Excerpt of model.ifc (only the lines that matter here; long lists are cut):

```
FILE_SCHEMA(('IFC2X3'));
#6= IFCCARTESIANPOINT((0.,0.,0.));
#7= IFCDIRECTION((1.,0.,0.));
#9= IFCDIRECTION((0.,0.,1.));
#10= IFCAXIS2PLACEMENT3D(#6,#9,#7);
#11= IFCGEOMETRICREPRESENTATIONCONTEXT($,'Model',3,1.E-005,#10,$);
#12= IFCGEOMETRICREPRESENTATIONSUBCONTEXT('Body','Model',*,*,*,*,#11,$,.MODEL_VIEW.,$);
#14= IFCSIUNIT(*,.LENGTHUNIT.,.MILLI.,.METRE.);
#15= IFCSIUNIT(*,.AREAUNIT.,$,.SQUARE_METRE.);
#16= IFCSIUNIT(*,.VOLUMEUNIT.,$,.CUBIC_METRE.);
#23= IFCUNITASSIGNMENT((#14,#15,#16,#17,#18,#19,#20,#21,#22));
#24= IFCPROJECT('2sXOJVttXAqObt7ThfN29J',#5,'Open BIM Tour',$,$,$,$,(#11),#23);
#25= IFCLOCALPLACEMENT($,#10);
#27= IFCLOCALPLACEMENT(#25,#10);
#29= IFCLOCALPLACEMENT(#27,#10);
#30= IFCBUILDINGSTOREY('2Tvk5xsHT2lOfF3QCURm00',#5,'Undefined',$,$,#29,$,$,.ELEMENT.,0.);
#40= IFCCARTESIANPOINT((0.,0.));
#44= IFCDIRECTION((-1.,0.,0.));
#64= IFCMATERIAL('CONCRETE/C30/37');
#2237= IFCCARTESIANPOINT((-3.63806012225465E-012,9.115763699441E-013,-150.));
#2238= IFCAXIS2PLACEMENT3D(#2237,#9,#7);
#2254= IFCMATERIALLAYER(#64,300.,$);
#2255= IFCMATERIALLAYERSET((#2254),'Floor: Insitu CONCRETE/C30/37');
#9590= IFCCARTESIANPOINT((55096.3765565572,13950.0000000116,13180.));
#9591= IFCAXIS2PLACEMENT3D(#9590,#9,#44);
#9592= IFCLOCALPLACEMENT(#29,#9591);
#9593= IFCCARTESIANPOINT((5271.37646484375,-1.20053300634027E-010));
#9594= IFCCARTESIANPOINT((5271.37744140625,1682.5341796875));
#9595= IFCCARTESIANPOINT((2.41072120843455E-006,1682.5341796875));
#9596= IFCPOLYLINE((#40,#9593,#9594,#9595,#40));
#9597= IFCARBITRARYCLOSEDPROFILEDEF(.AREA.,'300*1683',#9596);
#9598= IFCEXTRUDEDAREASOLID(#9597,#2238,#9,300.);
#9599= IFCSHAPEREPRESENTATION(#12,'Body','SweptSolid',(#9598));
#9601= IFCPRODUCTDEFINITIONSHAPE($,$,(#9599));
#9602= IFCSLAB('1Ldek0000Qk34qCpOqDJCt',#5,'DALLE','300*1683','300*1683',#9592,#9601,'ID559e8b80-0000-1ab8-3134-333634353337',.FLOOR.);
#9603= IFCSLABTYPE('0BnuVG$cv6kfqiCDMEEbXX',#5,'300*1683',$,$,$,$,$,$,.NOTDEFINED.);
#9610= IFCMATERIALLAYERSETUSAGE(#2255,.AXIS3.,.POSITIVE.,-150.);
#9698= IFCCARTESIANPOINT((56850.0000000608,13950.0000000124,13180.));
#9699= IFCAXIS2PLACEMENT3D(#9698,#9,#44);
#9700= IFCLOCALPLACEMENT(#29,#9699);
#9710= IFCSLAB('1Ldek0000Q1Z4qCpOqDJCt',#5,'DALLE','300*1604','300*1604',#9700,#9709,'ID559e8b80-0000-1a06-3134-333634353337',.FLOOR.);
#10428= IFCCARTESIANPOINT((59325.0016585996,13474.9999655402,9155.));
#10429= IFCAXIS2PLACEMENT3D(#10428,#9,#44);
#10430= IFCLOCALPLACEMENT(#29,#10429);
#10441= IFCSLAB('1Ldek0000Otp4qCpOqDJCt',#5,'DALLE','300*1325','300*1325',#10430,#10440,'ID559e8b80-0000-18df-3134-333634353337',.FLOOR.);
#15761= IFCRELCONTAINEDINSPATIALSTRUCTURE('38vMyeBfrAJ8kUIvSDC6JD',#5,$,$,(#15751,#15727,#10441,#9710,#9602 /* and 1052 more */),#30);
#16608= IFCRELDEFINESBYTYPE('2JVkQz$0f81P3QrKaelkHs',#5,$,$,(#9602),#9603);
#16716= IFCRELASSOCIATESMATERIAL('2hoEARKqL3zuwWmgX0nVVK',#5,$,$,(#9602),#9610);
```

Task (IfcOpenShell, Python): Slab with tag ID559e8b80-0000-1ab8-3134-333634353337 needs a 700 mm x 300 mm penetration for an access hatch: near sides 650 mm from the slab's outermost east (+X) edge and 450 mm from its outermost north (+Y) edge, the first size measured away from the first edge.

```python
import numpy as np
import ifcopenshell
import ifcopenshell.api.feature
import ifcopenshell.api.geometry
import ifcopenshell.api.root
import ifcopenshell.geom
import ifcopenshell.util.placement
import ifcopenshell.util.representation
import ifcopenshell.util.shape
import ifcopenshell.util.unit

model = ifcopenshell.open("model.ifc")
unit_scale = ifcopenshell.util.unit.calculate_unit_scale(model)
settings = ifcopenshell.geom.settings()


def volume(element):
    """Net volume in cubic metres, openings subtracted."""
    shape = ifcopenshell.geom.create_shape(settings, element)
    return ifcopenshell.util.shape.get_volume(shape.geometry)


slab = model.by_guid("1Ldek0000Qk34qCpOqDJCt")
before = volume(slab)

# Extent in the slab's own axes, in metres. The edges named are its -X and -Y sides.
slab_shape = ifcopenshell.geom.create_shape(settings, slab)
vertices = ifcopenshell.util.shape.get_vertices(slab_shape.geometry)
x_min, y_min, bottom = vertices.min(axis=0)
top = vertices[:, 2].max()

opening = ifcopenshell.api.root.create_entity(model, ifc_class="IfcOpeningElement", name="Access hatch opening")
context = ifcopenshell.util.representation.get_context(model, "Model", "Body", "MODEL_VIEW")
width, depth = 0.7, 0.3
outline = [(0.0, 0.0), (width, 0.0), (width, depth), (0.0, depth), (0.0, 0.0)]
# Overshoot both faces by 50 mm so the cut is clean.
shape = ifcopenshell.api.geometry.add_slab_representation(
    model, context=context, depth=top - bottom + 0.1, polyline=outline
)
ifcopenshell.api.geometry.assign_representation(model, product=opening, representation=shape)

matrix = ifcopenshell.util.placement.get_local_placement(slab.ObjectPlacement)
matrix[:, 3] = matrix @ np.append(np.array([x_min + 0.65, y_min + 0.45, bottom - 0.05]) / unit_scale, 1.0)
ifcopenshell.api.geometry.edit_object_placement(model, product=opening, matrix=matrix, is_si=False)
ifcopenshell.api.feature.add_feature(model, feature=opening, element=slab)

after = volume(slab)

print(f"slab volume {before:.3f} -> {after:.3f} m3")

model.write("model_edited.ifc")
```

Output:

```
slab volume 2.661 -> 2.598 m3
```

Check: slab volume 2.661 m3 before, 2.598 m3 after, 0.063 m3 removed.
